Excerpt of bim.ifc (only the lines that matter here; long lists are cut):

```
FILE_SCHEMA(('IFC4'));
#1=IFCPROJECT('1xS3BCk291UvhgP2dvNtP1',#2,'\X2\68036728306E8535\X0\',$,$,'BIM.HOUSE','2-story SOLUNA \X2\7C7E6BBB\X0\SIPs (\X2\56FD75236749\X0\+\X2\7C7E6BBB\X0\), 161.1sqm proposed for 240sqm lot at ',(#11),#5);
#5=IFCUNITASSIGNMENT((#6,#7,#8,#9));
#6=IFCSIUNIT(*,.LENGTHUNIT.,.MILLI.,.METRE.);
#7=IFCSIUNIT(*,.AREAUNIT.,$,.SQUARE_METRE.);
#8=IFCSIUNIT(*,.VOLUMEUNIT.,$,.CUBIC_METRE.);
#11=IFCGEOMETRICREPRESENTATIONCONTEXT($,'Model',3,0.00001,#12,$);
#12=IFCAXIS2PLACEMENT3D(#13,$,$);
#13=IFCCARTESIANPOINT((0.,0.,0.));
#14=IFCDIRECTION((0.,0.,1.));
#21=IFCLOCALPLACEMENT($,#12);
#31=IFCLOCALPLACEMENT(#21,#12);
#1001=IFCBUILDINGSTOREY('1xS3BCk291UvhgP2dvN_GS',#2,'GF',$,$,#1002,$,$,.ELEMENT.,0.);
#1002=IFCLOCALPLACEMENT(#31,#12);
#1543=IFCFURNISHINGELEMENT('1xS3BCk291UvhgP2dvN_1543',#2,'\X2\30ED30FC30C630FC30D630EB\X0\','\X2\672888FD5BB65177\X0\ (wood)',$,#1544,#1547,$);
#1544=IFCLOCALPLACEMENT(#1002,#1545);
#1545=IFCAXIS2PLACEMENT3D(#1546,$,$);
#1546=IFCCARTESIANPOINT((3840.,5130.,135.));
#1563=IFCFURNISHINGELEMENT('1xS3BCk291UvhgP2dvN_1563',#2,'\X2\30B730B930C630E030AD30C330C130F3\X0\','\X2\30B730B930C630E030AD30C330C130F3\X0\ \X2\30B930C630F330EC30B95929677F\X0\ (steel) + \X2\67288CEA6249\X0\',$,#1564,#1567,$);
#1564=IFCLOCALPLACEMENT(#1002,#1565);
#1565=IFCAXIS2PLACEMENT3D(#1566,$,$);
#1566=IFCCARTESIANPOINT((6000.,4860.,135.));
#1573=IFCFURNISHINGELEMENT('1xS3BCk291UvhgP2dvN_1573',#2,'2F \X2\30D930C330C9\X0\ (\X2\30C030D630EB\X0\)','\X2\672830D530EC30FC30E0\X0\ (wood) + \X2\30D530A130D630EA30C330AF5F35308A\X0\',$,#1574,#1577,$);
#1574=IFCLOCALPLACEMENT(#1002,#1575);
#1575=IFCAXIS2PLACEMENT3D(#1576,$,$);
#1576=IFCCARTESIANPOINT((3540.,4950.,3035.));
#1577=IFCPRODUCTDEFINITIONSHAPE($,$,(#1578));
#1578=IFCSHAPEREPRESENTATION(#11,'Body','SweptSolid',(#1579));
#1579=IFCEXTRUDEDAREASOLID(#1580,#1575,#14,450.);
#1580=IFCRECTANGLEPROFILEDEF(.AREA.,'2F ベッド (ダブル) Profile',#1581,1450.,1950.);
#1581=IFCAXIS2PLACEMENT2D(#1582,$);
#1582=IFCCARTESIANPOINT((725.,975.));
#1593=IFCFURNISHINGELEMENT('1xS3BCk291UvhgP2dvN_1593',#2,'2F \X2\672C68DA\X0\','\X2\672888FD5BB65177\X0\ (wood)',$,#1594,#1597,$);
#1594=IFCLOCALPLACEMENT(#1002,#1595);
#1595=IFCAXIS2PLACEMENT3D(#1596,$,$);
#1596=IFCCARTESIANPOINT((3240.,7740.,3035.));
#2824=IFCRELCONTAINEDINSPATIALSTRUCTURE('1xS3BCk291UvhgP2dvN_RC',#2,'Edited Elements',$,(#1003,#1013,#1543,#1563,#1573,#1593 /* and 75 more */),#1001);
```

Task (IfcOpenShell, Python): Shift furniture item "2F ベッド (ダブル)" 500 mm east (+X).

```python
import ifcopenshell
import ifcopenshell.api.geometry
import ifcopenshell.util.placement

model = ifcopenshell.open("bim.ifc")

item = model.by_guid("1xS3BCk291UvhgP2dvN_1573")
matrix = ifcopenshell.util.placement.get_local_placement(item.ObjectPlacement)
matrix[0, 3] += 500.0
ifcopenshell.api.geometry.edit_object_placement(model, product=item, matrix=matrix, is_si=False)

print(ifcopenshell.util.placement.get_local_placement(item.ObjectPlacement).round(3) + 0.0)

model.write("bim_updated.ifc")
```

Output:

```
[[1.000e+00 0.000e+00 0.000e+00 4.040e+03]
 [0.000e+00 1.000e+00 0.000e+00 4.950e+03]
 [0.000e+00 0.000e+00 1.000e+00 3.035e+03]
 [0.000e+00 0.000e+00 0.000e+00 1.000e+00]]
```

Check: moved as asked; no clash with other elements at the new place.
